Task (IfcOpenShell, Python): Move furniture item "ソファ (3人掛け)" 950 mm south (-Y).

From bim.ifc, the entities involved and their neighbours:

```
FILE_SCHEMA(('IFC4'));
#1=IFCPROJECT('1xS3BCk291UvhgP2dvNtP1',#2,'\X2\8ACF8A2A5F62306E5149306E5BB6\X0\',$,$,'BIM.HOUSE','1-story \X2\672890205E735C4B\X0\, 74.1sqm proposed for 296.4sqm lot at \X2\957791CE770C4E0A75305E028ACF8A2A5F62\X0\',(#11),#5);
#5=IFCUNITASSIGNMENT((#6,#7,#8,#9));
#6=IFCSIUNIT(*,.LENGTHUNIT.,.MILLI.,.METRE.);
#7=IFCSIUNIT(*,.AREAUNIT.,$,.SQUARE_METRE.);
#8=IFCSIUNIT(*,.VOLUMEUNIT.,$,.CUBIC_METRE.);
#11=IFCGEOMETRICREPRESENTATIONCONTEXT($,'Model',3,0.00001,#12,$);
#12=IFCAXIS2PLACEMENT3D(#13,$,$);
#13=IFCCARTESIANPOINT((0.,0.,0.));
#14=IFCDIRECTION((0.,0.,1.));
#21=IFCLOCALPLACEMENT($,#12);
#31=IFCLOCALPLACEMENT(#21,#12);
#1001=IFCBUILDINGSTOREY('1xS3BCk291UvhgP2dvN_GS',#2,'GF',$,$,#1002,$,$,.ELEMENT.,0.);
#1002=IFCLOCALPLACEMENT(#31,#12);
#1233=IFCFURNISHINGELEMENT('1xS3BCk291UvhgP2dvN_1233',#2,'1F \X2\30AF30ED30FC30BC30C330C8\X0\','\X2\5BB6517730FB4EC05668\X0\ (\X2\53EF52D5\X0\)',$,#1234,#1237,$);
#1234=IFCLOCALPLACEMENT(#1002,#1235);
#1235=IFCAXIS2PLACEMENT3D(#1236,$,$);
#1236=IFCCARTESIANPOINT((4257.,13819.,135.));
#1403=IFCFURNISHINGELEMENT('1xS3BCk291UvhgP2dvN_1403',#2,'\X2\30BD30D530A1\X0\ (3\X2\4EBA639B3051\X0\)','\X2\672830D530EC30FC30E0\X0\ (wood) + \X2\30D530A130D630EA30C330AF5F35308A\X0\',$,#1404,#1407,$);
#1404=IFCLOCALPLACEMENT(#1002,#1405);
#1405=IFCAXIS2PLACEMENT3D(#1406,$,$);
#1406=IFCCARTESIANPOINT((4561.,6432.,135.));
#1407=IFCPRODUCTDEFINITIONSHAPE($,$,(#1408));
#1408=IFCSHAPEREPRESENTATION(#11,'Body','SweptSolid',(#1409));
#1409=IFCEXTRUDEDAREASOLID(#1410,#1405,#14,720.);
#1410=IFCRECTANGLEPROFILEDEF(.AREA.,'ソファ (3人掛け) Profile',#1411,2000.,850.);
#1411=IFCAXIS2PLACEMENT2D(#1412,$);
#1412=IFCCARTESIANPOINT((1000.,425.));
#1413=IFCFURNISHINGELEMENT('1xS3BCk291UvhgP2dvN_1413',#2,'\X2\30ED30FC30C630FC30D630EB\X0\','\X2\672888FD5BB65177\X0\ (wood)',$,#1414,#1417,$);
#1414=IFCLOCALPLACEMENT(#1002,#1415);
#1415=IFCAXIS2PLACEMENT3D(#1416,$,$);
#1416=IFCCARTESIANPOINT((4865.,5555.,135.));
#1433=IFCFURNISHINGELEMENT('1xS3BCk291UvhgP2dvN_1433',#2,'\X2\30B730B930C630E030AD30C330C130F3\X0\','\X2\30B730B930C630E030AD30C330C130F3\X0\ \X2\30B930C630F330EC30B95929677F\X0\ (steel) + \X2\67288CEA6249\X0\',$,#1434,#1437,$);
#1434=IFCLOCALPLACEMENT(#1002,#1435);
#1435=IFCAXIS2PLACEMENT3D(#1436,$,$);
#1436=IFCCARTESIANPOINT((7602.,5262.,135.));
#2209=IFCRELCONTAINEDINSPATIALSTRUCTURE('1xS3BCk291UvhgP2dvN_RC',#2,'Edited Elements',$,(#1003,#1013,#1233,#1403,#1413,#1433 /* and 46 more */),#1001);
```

```python
import ifcopenshell
import ifcopenshell.api.geometry
import ifcopenshell.util.placement
import ifcopenshell.util.unit

model = ifcopenshell.open("bim.ifc")
unit_scale = ifcopenshell.util.unit.calculate_unit_scale(model)

item = model.by_guid("1xS3BCk291UvhgP2dvN_1403")
matrix = ifcopenshell.util.placement.get_local_placement(item.ObjectPlacement)
matrix[1, 3] -= 0.95 / unit_scale
ifcopenshell.api.geometry.edit_object_placement(model, product=item, matrix=matrix, is_si=False)

print(ifcopenshell.util.placement.get_local_placement(item.ObjectPlacement).round(3) + 0.0)

model.write("bim_edited.ifc")
```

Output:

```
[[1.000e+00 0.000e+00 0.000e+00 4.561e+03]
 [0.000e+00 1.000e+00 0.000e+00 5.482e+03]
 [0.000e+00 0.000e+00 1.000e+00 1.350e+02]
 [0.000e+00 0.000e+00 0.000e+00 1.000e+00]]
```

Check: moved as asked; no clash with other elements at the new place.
